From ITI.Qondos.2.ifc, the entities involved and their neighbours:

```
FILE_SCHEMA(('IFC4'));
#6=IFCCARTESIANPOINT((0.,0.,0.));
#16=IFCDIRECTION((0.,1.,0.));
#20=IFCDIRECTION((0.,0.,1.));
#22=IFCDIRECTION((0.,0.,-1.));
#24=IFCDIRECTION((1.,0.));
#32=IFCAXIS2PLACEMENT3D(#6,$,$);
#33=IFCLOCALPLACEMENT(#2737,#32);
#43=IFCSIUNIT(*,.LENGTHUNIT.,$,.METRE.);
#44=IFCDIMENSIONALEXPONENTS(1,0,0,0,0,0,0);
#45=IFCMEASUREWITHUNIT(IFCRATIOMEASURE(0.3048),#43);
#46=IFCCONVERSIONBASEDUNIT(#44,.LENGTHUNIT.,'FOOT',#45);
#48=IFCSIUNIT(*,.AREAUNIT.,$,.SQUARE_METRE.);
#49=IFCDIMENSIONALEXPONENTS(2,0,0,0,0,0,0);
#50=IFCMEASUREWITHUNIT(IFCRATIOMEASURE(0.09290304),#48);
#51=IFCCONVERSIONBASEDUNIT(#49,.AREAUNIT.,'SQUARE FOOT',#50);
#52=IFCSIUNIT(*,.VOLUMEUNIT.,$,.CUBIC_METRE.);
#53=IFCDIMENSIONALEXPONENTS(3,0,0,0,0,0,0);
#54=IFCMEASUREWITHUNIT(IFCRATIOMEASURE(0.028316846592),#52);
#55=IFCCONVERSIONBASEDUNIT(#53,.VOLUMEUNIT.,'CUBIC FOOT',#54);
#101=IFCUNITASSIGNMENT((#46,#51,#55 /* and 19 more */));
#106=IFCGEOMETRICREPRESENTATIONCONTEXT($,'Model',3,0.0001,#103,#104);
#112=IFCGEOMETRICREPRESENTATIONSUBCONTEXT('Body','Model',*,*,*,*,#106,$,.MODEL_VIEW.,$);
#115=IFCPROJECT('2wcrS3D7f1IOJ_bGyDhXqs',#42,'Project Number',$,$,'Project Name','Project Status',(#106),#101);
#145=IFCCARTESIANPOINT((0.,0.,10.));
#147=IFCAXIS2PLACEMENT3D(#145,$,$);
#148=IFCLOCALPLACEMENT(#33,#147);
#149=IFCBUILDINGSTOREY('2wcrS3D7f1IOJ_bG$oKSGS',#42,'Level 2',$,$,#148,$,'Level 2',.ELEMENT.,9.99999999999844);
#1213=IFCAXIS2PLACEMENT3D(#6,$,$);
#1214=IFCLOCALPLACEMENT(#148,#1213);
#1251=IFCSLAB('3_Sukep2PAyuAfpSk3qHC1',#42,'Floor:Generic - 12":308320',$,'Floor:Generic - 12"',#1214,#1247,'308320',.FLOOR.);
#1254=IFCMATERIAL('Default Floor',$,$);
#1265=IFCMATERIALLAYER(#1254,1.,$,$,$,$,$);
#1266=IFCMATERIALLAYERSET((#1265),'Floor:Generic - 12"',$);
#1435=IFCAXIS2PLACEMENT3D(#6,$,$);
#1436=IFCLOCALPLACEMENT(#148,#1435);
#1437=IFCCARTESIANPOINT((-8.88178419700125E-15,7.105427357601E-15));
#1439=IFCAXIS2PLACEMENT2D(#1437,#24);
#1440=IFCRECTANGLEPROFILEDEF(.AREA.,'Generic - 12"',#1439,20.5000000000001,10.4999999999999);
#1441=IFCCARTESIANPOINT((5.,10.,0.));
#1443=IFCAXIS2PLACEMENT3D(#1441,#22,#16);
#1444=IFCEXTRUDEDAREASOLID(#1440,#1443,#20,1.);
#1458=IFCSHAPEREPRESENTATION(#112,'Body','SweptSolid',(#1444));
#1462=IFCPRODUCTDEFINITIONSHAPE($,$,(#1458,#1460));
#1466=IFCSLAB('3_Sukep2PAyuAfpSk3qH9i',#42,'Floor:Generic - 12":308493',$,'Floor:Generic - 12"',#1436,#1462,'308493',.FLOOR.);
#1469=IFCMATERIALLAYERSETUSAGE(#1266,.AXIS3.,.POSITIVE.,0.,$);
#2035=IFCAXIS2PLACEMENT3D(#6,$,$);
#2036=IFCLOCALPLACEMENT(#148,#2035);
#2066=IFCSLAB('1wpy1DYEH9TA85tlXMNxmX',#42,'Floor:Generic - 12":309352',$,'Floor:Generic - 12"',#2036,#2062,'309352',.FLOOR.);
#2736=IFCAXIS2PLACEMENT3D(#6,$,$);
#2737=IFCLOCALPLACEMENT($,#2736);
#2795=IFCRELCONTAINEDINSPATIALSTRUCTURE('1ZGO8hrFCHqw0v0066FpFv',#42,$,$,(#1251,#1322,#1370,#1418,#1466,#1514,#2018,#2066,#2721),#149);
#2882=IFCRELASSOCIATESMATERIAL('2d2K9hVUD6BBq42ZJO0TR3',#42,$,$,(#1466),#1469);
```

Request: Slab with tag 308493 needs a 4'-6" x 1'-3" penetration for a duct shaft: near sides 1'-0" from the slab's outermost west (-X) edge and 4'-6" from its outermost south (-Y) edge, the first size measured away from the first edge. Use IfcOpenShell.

```python
import numpy as np
import ifcopenshell
import ifcopenshell.api.feature
import ifcopenshell.api.geometry
import ifcopenshell.api.root
import ifcopenshell.geom
import ifcopenshell.util.placement
import ifcopenshell.util.representation
import ifcopenshell.util.shape
import ifcopenshell.util.unit

model = ifcopenshell.open("ITI.Qondos.2.ifc")
unit_scale = ifcopenshell.util.unit.calculate_unit_scale(model)
settings = ifcopenshell.geom.settings()


def volume(element):
    """Net volume in cubic metres, openings subtracted."""
    shape = ifcopenshell.geom.create_shape(settings, element)
    return ifcopenshell.util.shape.get_volume(shape.geometry)


slab = model.by_guid("3_Sukep2PAyuAfpSk3qH9i")
before = volume(slab)

# Extent in the slab's own axes, in metres. The edges named are its -X and -Y sides.
slab_shape = ifcopenshell.geom.create_shape(settings, slab)
vertices = ifcopenshell.util.shape.get_vertices(slab_shape.geometry)
x_min, y_min, bottom = vertices.min(axis=0)
top = vertices[:, 2].max()

opening = ifcopenshell.api.root.create_entity(model, ifc_class="IfcOpeningElement", name="Duct shaft opening", predefined_type="OPENING")
context = ifcopenshell.util.representation.get_context(model, "Model", "Body", "MODEL_VIEW")
width, depth = 1.3716, 0.381
outline = [(0.0, 0.0), (width, 0.0), (width, depth), (0.0, depth), (0.0, 0.0)]
# Overshoot both faces by 50 mm so the cut is clean.
shape = ifcopenshell.api.geometry.add_slab_representation(
    model, context=context, depth=top - bottom + 0.1, polyline=outline
)
ifcopenshell.api.geometry.assign_representation(model, product=opening, representation=shape)

matrix = ifcopenshell.util.placement.get_local_placement(slab.ObjectPlacement)
matrix[:, 3] = matrix @ np.append(np.array([x_min + 0.3048, y_min + 1.3716, bottom - 0.05]) / unit_scale, 1.0)
ifcopenshell.api.geometry.edit_object_placement(model, product=opening, matrix=matrix, is_si=False)
ifcopenshell.api.feature.add_feature(model, feature=opening, element=slab)

after = volume(slab)

print(f"slab volume {before:.3f} -> {after:.3f} m3")

model.write("ITI.Qondos.2_rev.ifc")
```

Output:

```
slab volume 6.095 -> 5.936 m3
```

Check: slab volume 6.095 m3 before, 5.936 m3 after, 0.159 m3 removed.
